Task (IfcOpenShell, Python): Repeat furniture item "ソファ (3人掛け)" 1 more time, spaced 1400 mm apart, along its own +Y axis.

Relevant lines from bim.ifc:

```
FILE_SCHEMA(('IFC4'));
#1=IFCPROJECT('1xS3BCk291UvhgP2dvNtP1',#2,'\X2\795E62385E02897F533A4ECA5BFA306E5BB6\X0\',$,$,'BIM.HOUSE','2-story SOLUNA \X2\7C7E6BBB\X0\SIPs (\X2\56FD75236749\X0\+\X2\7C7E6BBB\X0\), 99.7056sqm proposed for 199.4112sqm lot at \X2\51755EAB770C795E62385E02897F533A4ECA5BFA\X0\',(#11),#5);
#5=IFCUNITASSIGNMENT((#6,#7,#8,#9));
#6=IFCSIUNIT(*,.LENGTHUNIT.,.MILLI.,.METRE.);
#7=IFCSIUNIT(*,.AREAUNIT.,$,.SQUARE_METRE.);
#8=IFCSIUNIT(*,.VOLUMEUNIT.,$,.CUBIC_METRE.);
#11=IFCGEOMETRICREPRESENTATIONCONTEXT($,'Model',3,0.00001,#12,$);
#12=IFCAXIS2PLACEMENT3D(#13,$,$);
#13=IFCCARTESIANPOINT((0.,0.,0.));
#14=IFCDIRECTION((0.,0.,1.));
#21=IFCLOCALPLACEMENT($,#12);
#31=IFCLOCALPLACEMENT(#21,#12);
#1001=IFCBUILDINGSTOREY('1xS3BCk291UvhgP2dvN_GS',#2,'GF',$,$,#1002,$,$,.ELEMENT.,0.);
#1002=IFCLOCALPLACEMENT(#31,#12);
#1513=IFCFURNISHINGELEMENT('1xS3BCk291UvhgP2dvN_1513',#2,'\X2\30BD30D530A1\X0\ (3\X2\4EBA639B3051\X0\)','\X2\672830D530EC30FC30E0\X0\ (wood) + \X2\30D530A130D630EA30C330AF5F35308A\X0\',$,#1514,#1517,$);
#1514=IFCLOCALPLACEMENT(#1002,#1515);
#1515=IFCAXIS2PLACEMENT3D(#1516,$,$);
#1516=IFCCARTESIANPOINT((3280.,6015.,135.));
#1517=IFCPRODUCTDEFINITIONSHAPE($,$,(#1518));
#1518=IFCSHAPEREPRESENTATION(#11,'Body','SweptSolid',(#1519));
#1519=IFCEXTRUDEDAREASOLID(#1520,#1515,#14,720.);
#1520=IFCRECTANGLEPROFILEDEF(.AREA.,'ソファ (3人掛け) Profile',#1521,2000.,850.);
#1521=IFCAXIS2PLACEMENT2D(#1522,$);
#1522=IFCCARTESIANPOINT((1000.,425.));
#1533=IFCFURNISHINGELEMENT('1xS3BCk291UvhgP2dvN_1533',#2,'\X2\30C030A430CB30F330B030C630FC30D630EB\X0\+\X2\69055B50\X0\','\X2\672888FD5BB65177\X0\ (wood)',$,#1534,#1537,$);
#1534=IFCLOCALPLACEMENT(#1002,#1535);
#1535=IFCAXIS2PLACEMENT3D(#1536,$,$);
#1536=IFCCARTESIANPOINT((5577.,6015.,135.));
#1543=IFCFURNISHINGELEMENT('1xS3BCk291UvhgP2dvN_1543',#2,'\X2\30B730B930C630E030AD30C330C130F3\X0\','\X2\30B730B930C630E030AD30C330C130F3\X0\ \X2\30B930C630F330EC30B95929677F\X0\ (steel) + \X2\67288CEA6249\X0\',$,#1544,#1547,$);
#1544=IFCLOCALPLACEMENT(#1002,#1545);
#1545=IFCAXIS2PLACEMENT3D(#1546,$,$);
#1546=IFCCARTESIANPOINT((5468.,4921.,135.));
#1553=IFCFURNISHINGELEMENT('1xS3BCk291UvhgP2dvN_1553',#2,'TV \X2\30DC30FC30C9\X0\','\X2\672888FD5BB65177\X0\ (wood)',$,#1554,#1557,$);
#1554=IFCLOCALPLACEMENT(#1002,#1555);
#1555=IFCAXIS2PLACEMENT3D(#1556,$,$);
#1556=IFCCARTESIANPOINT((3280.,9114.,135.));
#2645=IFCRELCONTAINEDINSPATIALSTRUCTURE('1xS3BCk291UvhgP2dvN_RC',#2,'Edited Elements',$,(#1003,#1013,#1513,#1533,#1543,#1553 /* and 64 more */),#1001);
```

```python
import ifcopenshell
import ifcopenshell.api.geometry
import ifcopenshell.api.root
import ifcopenshell.util.element
import ifcopenshell.util.placement
import ifcopenshell.util.unit

model = ifcopenshell.open("bim.ifc")
unit_scale = ifcopenshell.util.unit.calculate_unit_scale(model)


def reuse_history(source, copy):
    """copy_class also copies each property set's owner history, people and application; keep the originals."""
    for rel in copy.IsDefinedBy:
        if rel.is_a("IfcRelDefinesByProperties") and (history := rel.RelatingPropertyDefinition.OwnerHistory):
            rel.RelatingPropertyDefinition.OwnerHistory = source.OwnerHistory
            ifcopenshell.util.element.remove_deep2(model, history)


source = model.by_id(1513)
base = ifcopenshell.util.placement.get_local_placement(source.ObjectPlacement)
step = base[:3, 1] * 1.4 / unit_scale

for i in range(1, 2):
    copy = ifcopenshell.api.root.copy_class(model, product=source)
    copy.Representation = ifcopenshell.util.element.copy_deep(
        model, source.Representation, exclude=["IfcGeometricRepresentationContext", "IfcRepresentationMap"]
    )
    reuse_history(source, copy)
    matrix = base.copy()
    matrix[:3, 3] += i * step
    print("added at", matrix[:3, 3].round(3) + 0.0)
    ifcopenshell.api.geometry.edit_object_placement(model, product=copy, matrix=matrix, is_si=False)

model.write("bim-out.ifc")
```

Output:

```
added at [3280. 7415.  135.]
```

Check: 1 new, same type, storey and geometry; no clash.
